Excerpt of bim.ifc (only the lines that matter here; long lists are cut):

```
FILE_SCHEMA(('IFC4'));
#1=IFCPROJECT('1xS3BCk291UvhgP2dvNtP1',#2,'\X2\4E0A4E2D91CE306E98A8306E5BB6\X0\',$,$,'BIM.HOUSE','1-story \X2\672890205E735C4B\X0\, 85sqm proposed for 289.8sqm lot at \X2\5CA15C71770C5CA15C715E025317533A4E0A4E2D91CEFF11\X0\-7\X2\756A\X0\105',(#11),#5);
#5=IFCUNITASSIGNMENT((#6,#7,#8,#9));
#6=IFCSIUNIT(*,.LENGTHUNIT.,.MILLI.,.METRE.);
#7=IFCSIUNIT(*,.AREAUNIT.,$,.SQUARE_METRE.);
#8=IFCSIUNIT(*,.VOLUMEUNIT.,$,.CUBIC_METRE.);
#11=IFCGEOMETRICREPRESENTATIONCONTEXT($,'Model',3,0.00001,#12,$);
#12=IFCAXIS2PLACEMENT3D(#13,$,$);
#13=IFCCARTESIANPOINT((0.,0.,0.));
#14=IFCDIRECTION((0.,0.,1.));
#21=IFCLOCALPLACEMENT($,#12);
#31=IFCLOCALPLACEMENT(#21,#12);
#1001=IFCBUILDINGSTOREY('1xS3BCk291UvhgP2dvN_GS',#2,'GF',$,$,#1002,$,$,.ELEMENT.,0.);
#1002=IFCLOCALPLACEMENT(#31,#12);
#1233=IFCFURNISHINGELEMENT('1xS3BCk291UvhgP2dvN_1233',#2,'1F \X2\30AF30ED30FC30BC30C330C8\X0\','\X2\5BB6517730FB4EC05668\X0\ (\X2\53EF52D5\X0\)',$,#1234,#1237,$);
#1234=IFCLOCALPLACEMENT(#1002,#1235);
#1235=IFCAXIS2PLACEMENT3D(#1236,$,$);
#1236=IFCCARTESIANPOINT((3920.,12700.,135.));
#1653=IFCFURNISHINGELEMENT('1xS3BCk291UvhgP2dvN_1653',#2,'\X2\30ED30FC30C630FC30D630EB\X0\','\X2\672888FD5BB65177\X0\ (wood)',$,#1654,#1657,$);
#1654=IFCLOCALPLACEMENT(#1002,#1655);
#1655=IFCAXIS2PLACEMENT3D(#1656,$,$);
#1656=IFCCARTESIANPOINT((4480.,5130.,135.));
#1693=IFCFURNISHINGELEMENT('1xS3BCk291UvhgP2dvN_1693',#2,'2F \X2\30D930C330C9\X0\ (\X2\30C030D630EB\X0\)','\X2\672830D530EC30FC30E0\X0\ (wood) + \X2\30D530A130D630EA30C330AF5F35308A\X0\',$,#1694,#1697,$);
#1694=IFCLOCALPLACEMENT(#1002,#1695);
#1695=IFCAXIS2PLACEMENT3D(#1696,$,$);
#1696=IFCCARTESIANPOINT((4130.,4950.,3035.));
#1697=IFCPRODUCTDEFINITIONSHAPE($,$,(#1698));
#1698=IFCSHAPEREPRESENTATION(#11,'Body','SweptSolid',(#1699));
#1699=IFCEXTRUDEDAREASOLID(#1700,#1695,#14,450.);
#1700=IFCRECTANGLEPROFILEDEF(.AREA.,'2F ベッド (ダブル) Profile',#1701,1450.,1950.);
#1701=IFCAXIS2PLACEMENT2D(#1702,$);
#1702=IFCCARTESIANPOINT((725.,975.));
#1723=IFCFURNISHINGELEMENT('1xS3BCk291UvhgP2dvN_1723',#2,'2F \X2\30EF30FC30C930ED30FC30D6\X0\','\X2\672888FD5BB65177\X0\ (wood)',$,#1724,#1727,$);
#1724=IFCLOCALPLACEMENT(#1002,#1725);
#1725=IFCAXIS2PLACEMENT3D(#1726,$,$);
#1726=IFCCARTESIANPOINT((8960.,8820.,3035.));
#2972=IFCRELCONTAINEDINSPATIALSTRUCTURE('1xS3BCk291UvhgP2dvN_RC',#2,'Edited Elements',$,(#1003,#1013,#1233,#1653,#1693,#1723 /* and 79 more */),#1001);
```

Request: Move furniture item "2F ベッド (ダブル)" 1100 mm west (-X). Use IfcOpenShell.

```python
import ifcopenshell
import ifcopenshell.api.geometry
import ifcopenshell.util.placement
import ifcopenshell.util.unit

model = ifcopenshell.open("bim.ifc")
unit_scale = ifcopenshell.util.unit.calculate_unit_scale(model)

item = model.by_guid("1xS3BCk291UvhgP2dvN_1693")
matrix = ifcopenshell.util.placement.get_local_placement(item.ObjectPlacement)
matrix[0, 3] -= 1.1 / unit_scale
ifcopenshell.api.geometry.edit_object_placement(model, product=item, matrix=matrix, is_si=False)

print(ifcopenshell.util.placement.get_local_placement(item.ObjectPlacement).round(3) + 0.0)

model.write("bim_v2.ifc")
```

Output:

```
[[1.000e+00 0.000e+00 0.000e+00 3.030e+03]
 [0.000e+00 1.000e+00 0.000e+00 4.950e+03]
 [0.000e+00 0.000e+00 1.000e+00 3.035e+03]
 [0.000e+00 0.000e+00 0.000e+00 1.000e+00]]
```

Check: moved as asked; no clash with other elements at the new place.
